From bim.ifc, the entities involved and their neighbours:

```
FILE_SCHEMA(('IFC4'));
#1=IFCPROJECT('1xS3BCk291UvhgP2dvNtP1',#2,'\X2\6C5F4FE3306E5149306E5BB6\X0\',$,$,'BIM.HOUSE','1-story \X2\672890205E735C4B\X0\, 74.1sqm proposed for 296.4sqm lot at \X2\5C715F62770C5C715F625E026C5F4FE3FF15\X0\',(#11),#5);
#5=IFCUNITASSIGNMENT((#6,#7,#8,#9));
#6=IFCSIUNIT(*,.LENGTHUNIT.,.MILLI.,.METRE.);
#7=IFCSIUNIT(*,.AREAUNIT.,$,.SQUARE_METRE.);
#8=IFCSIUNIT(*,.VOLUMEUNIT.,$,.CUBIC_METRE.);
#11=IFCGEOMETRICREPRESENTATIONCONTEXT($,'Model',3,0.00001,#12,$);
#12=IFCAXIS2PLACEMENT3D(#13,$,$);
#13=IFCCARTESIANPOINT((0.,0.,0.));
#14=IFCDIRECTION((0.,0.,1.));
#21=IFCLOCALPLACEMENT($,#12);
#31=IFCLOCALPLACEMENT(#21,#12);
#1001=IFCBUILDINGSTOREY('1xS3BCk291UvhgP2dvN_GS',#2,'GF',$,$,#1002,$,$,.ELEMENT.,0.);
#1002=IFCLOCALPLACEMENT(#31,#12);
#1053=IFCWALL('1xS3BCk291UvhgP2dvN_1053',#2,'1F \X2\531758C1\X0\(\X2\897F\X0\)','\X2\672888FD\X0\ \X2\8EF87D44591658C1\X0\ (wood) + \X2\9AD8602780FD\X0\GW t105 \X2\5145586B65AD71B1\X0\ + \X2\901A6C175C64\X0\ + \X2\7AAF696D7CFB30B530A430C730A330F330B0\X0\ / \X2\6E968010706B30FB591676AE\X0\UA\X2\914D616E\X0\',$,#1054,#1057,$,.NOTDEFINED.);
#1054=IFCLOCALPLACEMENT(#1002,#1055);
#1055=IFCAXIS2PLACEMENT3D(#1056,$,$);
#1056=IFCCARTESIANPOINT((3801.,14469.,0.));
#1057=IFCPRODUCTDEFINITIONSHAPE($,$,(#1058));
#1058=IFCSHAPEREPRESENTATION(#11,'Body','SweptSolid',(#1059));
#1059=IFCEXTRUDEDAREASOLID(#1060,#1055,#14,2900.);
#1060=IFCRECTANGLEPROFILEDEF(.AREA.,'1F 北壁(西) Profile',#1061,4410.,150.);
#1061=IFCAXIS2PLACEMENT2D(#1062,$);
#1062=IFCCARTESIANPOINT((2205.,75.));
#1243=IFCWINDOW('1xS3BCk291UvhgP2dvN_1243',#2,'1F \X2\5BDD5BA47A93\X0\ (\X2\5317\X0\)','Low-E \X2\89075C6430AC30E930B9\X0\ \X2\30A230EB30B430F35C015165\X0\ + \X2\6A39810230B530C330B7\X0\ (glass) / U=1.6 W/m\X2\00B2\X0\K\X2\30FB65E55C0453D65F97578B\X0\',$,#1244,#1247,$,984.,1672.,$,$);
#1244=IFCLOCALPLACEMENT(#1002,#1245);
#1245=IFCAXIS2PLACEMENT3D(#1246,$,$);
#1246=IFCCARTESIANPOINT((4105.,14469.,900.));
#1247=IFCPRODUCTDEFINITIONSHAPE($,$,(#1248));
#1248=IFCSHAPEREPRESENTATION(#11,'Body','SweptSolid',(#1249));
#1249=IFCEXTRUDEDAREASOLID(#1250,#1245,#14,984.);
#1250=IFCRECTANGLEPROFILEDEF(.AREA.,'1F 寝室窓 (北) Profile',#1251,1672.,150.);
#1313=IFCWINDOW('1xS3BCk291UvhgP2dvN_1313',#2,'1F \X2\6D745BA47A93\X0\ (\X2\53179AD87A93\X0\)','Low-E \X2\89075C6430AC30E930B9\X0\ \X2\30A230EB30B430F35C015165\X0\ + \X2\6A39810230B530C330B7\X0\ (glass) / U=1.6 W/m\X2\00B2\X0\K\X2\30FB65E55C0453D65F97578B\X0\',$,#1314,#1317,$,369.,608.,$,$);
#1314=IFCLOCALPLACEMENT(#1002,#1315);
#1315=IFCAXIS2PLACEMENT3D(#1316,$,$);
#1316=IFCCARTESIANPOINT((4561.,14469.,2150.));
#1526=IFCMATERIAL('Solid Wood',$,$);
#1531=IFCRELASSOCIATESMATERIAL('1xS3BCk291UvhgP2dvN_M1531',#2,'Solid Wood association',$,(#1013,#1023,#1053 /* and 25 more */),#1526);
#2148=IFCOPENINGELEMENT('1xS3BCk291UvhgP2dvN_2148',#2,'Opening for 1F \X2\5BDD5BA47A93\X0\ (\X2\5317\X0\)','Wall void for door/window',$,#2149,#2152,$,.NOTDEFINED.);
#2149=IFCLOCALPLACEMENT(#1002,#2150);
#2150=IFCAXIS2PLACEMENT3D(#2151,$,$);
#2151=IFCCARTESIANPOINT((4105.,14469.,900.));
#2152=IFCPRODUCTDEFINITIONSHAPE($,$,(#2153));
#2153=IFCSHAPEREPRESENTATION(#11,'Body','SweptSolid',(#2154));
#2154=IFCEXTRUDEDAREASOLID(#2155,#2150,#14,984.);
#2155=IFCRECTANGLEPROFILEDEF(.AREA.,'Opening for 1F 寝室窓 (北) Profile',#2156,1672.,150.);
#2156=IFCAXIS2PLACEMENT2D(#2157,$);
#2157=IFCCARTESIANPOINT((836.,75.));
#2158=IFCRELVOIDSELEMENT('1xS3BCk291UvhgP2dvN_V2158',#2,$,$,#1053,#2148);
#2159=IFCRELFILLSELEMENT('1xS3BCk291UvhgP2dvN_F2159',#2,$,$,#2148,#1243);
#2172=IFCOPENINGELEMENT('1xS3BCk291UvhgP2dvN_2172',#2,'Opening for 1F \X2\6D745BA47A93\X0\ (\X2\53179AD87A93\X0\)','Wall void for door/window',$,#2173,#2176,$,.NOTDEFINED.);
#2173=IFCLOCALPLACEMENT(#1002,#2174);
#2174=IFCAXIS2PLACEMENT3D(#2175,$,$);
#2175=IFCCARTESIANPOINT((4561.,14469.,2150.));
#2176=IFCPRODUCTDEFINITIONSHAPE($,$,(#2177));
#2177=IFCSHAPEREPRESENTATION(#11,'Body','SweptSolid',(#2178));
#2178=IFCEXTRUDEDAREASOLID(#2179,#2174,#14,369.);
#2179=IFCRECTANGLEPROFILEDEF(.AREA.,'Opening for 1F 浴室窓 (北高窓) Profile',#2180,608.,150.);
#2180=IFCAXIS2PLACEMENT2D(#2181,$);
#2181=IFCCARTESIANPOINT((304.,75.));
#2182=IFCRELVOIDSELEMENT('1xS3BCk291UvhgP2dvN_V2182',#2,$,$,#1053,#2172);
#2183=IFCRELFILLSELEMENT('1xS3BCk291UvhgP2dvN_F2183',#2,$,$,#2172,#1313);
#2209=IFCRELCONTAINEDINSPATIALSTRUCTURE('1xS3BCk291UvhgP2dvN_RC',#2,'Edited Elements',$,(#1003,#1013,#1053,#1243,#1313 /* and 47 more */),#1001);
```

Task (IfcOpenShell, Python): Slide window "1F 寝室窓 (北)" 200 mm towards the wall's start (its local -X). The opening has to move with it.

```python
import ifcopenshell
import ifcopenshell.api.geometry
import ifcopenshell.util.placement

model = ifcopenshell.open("bim.ifc")

window = model.by_guid("1xS3BCk291UvhgP2dvN_1243")
opening = window.FillsVoids[0].RelatingOpeningElement
wall = opening.VoidsElements[0].RelatingBuildingElement

wall_matrix = ifcopenshell.util.placement.get_local_placement(wall.ObjectPlacement)
shift = wall_matrix[:3, 0] * -200.0
before = ifcopenshell.util.placement.get_local_placement(window.ObjectPlacement)[:3, 3].copy()

# The window is not placed relative to its opening, so move both.
for product in (opening, window):
    matrix = ifcopenshell.util.placement.get_local_placement(product.ObjectPlacement)
    matrix[:3, 3] += shift
    ifcopenshell.api.geometry.edit_object_placement(model, product=product, matrix=matrix, is_si=False)

after = ifcopenshell.util.placement.get_local_placement(window.ObjectPlacement)[:3, 3]
print("window moved by", (after - before).round(3) + 0.0)

model.write("bim_v2.ifc")
```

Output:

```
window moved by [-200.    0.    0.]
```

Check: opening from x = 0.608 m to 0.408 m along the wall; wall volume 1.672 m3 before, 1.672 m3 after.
